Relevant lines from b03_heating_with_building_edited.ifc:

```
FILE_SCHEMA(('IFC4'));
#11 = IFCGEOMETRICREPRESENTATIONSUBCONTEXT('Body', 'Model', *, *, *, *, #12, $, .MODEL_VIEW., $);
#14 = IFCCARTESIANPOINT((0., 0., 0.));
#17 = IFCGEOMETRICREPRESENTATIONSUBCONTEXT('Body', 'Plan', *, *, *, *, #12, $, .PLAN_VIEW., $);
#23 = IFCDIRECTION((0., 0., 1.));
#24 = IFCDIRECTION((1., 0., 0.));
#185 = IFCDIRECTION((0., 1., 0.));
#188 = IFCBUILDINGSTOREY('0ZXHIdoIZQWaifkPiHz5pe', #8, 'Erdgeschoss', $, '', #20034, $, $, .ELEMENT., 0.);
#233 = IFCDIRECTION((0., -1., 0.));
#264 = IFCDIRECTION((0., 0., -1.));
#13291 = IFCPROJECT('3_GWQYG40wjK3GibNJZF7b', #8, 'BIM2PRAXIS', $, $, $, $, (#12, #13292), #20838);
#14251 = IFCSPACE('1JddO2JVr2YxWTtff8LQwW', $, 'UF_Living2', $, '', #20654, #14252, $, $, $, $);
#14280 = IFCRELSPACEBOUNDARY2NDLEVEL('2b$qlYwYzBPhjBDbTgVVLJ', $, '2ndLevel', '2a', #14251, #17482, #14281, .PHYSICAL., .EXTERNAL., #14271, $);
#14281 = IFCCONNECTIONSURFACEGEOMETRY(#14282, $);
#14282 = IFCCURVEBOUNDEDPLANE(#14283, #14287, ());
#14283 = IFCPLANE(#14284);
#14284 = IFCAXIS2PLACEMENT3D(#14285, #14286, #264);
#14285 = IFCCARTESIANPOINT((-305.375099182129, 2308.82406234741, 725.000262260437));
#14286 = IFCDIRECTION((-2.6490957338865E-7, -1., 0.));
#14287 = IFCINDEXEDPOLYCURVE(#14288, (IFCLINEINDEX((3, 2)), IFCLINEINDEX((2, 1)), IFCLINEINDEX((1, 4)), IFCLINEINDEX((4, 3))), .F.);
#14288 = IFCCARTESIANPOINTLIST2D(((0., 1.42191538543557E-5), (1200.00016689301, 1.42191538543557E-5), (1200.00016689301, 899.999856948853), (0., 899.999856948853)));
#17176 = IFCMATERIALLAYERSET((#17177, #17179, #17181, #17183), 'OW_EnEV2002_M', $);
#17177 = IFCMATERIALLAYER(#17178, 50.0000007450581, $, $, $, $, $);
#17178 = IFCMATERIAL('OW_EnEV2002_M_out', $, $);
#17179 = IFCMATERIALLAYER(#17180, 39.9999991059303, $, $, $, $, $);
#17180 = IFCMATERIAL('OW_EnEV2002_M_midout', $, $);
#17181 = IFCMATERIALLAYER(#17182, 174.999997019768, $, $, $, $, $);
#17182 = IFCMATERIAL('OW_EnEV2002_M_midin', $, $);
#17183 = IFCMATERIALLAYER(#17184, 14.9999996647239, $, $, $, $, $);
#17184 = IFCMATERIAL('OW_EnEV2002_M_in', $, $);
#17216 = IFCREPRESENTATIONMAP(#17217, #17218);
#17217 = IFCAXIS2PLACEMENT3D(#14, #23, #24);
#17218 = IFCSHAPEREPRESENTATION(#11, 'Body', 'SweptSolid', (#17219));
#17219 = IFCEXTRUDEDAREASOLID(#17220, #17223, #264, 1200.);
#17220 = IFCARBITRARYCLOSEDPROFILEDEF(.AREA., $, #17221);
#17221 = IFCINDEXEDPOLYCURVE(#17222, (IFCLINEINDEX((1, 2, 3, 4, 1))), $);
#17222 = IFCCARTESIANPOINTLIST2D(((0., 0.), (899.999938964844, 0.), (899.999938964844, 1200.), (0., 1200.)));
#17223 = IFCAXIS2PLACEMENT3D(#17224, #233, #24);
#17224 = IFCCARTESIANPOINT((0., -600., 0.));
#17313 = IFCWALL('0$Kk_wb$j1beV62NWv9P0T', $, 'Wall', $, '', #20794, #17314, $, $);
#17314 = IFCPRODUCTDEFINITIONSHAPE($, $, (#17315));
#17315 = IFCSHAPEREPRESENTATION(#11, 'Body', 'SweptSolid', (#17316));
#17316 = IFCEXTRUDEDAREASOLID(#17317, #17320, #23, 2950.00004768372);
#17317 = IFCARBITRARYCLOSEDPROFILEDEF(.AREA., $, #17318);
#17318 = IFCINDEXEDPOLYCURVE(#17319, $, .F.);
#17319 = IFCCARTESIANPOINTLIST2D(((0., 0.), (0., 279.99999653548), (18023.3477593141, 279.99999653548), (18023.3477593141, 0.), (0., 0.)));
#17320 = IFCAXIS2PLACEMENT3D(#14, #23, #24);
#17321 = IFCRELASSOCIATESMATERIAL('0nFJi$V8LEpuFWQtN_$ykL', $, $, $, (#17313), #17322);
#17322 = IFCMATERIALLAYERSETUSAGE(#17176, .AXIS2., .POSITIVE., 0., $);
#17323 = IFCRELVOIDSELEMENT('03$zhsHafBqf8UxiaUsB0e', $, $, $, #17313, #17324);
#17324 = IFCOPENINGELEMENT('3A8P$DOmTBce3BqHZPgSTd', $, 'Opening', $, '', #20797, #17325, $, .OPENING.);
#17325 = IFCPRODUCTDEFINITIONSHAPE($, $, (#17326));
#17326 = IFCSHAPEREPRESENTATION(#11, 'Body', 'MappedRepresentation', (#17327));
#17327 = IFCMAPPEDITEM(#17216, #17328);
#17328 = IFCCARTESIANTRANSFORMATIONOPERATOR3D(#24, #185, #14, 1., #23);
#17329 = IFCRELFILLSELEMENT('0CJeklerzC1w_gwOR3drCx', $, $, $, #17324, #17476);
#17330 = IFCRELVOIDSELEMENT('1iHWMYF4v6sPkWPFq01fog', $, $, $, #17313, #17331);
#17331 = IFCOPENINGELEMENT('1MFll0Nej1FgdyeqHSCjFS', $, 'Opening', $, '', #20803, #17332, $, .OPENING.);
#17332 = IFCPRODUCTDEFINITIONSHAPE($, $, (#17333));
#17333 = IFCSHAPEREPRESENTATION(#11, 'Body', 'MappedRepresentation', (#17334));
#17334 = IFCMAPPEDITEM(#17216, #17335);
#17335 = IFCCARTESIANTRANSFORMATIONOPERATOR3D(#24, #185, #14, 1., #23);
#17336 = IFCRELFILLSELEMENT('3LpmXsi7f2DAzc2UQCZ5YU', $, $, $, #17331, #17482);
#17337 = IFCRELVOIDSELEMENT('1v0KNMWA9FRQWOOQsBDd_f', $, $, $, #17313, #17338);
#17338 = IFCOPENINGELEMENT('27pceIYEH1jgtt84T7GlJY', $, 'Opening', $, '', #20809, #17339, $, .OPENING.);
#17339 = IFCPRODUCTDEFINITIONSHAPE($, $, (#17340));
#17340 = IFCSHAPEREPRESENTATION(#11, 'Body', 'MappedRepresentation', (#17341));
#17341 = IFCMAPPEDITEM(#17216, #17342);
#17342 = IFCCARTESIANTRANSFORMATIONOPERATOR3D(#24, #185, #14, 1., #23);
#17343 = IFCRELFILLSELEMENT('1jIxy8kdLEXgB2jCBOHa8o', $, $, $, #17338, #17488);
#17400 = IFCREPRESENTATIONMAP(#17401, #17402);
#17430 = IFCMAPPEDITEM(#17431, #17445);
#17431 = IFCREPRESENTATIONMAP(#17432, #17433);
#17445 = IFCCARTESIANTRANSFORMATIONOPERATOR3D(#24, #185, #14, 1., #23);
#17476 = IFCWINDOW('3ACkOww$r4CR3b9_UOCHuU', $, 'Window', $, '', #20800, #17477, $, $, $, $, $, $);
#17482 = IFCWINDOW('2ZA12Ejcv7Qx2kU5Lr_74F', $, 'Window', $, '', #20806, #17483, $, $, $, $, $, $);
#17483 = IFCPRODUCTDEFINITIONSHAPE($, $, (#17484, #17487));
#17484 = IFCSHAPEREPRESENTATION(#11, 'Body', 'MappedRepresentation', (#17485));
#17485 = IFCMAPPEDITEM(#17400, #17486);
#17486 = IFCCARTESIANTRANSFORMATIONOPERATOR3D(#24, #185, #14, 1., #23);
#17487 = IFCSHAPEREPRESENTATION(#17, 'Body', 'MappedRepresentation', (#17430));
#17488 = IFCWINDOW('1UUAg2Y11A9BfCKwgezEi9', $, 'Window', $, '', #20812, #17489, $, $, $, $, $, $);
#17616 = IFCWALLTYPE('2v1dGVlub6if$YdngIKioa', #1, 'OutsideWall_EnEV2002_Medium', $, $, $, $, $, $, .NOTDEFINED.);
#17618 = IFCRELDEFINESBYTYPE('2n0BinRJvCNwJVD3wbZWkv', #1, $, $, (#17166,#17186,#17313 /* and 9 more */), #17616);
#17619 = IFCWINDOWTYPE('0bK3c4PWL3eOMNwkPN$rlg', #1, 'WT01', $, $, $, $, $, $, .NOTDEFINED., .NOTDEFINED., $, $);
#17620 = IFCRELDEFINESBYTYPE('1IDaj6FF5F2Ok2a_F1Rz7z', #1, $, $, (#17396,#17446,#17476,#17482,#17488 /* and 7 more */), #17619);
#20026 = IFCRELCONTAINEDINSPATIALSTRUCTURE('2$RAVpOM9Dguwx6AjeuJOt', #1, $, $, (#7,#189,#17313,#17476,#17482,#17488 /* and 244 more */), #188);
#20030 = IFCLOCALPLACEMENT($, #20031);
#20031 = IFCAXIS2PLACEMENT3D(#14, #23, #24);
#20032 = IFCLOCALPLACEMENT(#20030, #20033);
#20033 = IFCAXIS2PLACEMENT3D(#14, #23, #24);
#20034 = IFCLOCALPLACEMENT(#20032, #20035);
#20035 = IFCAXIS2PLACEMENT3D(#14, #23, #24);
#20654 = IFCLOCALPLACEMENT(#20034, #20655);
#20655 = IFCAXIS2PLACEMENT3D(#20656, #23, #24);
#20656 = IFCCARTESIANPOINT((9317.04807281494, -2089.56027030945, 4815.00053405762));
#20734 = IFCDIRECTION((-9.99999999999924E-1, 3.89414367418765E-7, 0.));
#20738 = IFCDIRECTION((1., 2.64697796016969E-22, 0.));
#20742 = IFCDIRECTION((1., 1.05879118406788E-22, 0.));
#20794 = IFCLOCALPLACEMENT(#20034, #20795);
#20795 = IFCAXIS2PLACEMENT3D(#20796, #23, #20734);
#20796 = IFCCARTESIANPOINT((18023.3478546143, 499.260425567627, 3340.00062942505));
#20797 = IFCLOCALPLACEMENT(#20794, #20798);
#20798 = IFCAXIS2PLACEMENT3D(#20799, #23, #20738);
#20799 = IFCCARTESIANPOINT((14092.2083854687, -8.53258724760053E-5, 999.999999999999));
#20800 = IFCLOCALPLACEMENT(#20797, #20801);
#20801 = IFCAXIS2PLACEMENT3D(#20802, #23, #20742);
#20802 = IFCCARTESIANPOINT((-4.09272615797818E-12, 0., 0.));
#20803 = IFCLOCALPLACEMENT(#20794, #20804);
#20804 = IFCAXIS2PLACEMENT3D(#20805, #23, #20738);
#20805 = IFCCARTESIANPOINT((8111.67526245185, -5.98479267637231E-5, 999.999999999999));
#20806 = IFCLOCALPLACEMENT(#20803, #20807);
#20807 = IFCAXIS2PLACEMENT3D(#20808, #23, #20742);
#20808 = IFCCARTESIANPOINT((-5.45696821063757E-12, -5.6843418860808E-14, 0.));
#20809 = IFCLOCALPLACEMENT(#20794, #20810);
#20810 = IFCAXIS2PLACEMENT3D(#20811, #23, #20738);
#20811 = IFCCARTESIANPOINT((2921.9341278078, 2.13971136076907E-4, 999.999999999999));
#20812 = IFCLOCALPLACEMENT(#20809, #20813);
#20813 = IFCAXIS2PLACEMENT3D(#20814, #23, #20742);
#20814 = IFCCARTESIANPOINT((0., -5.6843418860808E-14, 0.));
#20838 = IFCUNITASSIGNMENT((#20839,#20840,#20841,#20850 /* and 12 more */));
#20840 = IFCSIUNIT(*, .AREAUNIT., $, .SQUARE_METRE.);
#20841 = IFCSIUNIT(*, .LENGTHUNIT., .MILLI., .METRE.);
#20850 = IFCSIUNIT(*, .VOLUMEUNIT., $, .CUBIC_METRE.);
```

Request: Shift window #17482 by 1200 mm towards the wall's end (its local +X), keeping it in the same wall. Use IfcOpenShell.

```python
import numpy as np
import ifcopenshell
import ifcopenshell.api.geometry
import ifcopenshell.util.placement
import ifcopenshell.util.unit

model = ifcopenshell.open("b03_heating_with_building_edited.ifc")
unit_scale = ifcopenshell.util.unit.calculate_unit_scale(model)

window = model.by_id(17482)
opening = window.FillsVoids[0].RelatingOpeningElement
wall = opening.VoidsElements[0].RelatingBuildingElement

wall_matrix = ifcopenshell.util.placement.get_local_placement(wall.ObjectPlacement)
shift = wall_matrix[:3, 0] * 1.2 / unit_scale
before = ifcopenshell.util.placement.get_local_placement(window.ObjectPlacement)[:3, 3].copy()

# The window is placed relative to its opening, so it follows when the opening moves.
matrix = ifcopenshell.util.placement.get_local_placement(opening.ObjectPlacement)
matrix[:3, 3] += shift
ifcopenshell.api.geometry.edit_object_placement(
    model, product=opening, matrix=matrix, is_si=False, should_transform_children=True
)

# Space boundary surfaces are stored in each space's coordinates; move them too.
for rel in window.ProvidesBoundaries:
    if not rel.ConnectionGeometry:
        continue
    surface = rel.ConnectionGeometry.SurfaceOnRelatingElement.BasisSurface
    space_matrix = ifcopenshell.util.placement.get_local_placement(rel.RelatingSpace.ObjectPlacement)
    point = np.array(surface.Position.Location.Coordinates) + space_matrix[:3, :3].T @ shift
    surface.Position = model.createIfcAxis2Placement3D(
        model.createIfcCartesianPoint(point.tolist()), surface.Position.Axis, surface.Position.RefDirection
    )

after = ifcopenshell.util.placement.get_local_placement(window.ObjectPlacement)[:3, 3]
print("window moved by", (after - before).round(3) + 0.0)

model.write("b03_heating_with_building_edited_v2.ifc")
```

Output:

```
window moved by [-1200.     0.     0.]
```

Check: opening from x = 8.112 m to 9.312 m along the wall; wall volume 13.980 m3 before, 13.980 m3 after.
